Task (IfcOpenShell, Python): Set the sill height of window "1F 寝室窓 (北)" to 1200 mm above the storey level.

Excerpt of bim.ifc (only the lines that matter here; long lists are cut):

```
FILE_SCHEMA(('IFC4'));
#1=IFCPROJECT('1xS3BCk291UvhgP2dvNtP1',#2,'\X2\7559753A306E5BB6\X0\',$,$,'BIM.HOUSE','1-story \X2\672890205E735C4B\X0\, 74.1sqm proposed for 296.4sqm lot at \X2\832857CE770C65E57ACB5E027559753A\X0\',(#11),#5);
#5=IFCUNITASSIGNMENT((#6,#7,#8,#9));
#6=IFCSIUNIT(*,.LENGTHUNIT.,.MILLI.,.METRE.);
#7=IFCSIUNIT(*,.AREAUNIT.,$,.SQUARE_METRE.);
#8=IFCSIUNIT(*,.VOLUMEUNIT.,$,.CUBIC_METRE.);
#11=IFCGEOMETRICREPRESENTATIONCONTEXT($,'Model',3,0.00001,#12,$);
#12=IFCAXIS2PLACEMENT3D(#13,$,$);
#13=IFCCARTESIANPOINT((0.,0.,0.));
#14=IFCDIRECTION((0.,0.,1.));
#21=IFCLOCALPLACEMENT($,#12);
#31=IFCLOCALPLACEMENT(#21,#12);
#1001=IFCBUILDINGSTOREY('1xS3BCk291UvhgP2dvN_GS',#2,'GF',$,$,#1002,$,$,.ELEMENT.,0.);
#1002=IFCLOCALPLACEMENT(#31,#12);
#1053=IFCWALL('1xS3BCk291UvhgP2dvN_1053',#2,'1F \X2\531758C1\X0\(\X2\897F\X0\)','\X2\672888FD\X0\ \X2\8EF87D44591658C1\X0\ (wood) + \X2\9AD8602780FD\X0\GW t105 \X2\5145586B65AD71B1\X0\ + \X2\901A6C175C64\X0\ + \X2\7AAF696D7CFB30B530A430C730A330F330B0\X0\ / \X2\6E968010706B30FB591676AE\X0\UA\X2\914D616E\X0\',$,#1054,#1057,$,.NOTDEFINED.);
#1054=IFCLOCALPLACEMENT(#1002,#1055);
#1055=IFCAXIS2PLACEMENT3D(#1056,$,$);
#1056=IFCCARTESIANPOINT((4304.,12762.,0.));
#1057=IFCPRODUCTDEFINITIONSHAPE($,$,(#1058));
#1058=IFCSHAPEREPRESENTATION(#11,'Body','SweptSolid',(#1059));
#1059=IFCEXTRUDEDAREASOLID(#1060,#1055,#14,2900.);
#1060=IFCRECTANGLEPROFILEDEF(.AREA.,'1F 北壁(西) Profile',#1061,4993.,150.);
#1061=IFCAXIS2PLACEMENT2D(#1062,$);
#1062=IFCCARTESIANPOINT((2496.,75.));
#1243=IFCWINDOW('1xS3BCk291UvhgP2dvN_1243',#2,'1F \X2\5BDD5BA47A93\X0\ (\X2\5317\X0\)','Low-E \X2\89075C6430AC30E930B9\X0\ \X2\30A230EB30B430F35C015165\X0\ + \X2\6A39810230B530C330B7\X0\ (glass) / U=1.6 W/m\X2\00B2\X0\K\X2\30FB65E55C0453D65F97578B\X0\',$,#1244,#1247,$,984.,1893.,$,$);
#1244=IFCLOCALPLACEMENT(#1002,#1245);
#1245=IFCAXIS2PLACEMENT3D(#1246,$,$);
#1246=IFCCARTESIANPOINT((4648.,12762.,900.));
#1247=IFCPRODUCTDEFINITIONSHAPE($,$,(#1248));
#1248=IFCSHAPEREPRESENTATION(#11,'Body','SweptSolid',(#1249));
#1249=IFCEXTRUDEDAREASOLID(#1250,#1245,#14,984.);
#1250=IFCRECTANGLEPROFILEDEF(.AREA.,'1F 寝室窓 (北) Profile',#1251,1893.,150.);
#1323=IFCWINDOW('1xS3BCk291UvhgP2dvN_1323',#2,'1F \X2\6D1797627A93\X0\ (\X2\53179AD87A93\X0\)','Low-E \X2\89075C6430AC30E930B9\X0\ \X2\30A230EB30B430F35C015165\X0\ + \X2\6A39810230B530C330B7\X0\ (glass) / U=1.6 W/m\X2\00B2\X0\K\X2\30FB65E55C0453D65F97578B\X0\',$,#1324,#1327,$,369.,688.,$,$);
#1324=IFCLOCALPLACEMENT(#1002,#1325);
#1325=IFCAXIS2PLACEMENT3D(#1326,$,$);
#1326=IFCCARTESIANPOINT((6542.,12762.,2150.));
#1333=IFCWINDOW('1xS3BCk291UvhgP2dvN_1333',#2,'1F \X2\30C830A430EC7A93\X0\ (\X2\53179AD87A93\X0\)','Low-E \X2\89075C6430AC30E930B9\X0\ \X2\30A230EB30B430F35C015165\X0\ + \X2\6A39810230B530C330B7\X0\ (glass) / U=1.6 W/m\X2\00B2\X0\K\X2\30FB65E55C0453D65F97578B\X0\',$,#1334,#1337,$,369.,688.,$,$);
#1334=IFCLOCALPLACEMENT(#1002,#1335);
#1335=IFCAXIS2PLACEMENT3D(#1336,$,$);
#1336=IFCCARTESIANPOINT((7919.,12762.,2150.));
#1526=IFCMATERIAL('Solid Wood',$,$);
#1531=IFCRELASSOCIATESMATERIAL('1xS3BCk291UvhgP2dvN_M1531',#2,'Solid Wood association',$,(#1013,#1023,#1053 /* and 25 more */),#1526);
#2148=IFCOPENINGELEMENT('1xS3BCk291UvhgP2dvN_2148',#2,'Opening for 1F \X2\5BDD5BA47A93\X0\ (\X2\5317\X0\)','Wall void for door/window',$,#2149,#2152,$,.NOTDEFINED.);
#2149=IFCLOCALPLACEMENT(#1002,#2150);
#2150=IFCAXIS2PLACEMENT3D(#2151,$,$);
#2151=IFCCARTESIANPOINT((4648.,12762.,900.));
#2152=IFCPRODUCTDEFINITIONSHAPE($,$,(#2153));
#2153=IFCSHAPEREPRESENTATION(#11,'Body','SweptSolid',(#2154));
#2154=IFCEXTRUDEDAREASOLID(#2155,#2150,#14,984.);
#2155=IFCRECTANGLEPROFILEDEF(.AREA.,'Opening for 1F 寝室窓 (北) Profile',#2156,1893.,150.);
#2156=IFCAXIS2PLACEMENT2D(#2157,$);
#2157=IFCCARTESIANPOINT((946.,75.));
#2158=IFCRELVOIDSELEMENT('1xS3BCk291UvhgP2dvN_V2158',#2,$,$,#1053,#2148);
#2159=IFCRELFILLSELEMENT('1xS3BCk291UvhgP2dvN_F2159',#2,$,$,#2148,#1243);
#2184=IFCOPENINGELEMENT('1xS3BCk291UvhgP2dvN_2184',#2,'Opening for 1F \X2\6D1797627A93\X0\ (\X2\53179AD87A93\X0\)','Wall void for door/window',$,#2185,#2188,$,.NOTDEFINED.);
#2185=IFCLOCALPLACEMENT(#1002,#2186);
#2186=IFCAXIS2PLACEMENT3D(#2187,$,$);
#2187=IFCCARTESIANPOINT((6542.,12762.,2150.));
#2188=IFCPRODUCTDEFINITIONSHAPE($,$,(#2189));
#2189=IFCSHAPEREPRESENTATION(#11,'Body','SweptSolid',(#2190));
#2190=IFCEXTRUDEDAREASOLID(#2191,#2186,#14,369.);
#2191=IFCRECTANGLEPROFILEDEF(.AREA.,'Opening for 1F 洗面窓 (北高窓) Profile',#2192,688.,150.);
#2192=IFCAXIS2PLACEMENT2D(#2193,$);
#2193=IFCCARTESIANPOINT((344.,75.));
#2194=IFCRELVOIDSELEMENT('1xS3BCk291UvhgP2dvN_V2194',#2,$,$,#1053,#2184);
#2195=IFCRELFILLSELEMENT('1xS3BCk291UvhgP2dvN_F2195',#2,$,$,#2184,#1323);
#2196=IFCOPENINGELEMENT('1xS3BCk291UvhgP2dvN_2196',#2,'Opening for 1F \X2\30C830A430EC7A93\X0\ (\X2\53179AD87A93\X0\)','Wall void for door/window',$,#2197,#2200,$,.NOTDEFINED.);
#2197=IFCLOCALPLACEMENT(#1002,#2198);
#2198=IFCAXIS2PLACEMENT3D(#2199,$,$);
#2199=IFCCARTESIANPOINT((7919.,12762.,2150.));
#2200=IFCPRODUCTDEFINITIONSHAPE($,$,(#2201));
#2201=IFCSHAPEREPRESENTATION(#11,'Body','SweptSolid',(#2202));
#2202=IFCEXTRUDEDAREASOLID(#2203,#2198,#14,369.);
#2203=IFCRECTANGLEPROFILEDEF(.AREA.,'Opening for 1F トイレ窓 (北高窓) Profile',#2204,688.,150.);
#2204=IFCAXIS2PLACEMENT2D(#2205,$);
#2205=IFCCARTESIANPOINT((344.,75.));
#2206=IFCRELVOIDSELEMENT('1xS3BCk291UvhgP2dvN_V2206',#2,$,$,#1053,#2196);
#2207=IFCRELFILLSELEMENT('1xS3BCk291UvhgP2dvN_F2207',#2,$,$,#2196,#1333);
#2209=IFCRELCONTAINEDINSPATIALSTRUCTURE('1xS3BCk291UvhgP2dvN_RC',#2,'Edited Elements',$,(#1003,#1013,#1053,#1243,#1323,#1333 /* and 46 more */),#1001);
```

```python
import numpy as np
import ifcopenshell
import ifcopenshell.api.geometry
import ifcopenshell.geom
import ifcopenshell.util.element
import ifcopenshell.util.placement
import ifcopenshell.util.shape
import ifcopenshell.util.unit

model = ifcopenshell.open("bim.ifc")
unit_scale = ifcopenshell.util.unit.calculate_unit_scale(model)

window = model.by_guid("1xS3BCk291UvhgP2dvN_1243")
opening = window.FillsVoids[0].RelatingOpeningElement
storey = ifcopenshell.util.element.get_container(window, ifc_class="IfcBuildingStorey")
level = ifcopenshell.util.placement.get_local_placement(storey.ObjectPlacement)[2, 3]

# The opening's origin need not be at the sill, so measure its lowest point.
shape = ifcopenshell.geom.create_shape(ifcopenshell.geom.settings(), opening)
bottom = ifcopenshell.util.shape.get_shape_bottom_elevation(shape, shape.geometry) / unit_scale
dz = level + 1200.0 - bottom

shift = np.array([0.0, 0.0, dz])
# The window is not placed relative to its opening, so move both.
for product in (opening, window):
    matrix = ifcopenshell.util.placement.get_local_placement(product.ObjectPlacement)
    matrix[:3, 3] += shift
    ifcopenshell.api.geometry.edit_object_placement(model, product=product, matrix=matrix, is_si=False)

print(f"moved by {dz * unit_scale:+.3f} m")

model.write("bim_updated.ifc")
```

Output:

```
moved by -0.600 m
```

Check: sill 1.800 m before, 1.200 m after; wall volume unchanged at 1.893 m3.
